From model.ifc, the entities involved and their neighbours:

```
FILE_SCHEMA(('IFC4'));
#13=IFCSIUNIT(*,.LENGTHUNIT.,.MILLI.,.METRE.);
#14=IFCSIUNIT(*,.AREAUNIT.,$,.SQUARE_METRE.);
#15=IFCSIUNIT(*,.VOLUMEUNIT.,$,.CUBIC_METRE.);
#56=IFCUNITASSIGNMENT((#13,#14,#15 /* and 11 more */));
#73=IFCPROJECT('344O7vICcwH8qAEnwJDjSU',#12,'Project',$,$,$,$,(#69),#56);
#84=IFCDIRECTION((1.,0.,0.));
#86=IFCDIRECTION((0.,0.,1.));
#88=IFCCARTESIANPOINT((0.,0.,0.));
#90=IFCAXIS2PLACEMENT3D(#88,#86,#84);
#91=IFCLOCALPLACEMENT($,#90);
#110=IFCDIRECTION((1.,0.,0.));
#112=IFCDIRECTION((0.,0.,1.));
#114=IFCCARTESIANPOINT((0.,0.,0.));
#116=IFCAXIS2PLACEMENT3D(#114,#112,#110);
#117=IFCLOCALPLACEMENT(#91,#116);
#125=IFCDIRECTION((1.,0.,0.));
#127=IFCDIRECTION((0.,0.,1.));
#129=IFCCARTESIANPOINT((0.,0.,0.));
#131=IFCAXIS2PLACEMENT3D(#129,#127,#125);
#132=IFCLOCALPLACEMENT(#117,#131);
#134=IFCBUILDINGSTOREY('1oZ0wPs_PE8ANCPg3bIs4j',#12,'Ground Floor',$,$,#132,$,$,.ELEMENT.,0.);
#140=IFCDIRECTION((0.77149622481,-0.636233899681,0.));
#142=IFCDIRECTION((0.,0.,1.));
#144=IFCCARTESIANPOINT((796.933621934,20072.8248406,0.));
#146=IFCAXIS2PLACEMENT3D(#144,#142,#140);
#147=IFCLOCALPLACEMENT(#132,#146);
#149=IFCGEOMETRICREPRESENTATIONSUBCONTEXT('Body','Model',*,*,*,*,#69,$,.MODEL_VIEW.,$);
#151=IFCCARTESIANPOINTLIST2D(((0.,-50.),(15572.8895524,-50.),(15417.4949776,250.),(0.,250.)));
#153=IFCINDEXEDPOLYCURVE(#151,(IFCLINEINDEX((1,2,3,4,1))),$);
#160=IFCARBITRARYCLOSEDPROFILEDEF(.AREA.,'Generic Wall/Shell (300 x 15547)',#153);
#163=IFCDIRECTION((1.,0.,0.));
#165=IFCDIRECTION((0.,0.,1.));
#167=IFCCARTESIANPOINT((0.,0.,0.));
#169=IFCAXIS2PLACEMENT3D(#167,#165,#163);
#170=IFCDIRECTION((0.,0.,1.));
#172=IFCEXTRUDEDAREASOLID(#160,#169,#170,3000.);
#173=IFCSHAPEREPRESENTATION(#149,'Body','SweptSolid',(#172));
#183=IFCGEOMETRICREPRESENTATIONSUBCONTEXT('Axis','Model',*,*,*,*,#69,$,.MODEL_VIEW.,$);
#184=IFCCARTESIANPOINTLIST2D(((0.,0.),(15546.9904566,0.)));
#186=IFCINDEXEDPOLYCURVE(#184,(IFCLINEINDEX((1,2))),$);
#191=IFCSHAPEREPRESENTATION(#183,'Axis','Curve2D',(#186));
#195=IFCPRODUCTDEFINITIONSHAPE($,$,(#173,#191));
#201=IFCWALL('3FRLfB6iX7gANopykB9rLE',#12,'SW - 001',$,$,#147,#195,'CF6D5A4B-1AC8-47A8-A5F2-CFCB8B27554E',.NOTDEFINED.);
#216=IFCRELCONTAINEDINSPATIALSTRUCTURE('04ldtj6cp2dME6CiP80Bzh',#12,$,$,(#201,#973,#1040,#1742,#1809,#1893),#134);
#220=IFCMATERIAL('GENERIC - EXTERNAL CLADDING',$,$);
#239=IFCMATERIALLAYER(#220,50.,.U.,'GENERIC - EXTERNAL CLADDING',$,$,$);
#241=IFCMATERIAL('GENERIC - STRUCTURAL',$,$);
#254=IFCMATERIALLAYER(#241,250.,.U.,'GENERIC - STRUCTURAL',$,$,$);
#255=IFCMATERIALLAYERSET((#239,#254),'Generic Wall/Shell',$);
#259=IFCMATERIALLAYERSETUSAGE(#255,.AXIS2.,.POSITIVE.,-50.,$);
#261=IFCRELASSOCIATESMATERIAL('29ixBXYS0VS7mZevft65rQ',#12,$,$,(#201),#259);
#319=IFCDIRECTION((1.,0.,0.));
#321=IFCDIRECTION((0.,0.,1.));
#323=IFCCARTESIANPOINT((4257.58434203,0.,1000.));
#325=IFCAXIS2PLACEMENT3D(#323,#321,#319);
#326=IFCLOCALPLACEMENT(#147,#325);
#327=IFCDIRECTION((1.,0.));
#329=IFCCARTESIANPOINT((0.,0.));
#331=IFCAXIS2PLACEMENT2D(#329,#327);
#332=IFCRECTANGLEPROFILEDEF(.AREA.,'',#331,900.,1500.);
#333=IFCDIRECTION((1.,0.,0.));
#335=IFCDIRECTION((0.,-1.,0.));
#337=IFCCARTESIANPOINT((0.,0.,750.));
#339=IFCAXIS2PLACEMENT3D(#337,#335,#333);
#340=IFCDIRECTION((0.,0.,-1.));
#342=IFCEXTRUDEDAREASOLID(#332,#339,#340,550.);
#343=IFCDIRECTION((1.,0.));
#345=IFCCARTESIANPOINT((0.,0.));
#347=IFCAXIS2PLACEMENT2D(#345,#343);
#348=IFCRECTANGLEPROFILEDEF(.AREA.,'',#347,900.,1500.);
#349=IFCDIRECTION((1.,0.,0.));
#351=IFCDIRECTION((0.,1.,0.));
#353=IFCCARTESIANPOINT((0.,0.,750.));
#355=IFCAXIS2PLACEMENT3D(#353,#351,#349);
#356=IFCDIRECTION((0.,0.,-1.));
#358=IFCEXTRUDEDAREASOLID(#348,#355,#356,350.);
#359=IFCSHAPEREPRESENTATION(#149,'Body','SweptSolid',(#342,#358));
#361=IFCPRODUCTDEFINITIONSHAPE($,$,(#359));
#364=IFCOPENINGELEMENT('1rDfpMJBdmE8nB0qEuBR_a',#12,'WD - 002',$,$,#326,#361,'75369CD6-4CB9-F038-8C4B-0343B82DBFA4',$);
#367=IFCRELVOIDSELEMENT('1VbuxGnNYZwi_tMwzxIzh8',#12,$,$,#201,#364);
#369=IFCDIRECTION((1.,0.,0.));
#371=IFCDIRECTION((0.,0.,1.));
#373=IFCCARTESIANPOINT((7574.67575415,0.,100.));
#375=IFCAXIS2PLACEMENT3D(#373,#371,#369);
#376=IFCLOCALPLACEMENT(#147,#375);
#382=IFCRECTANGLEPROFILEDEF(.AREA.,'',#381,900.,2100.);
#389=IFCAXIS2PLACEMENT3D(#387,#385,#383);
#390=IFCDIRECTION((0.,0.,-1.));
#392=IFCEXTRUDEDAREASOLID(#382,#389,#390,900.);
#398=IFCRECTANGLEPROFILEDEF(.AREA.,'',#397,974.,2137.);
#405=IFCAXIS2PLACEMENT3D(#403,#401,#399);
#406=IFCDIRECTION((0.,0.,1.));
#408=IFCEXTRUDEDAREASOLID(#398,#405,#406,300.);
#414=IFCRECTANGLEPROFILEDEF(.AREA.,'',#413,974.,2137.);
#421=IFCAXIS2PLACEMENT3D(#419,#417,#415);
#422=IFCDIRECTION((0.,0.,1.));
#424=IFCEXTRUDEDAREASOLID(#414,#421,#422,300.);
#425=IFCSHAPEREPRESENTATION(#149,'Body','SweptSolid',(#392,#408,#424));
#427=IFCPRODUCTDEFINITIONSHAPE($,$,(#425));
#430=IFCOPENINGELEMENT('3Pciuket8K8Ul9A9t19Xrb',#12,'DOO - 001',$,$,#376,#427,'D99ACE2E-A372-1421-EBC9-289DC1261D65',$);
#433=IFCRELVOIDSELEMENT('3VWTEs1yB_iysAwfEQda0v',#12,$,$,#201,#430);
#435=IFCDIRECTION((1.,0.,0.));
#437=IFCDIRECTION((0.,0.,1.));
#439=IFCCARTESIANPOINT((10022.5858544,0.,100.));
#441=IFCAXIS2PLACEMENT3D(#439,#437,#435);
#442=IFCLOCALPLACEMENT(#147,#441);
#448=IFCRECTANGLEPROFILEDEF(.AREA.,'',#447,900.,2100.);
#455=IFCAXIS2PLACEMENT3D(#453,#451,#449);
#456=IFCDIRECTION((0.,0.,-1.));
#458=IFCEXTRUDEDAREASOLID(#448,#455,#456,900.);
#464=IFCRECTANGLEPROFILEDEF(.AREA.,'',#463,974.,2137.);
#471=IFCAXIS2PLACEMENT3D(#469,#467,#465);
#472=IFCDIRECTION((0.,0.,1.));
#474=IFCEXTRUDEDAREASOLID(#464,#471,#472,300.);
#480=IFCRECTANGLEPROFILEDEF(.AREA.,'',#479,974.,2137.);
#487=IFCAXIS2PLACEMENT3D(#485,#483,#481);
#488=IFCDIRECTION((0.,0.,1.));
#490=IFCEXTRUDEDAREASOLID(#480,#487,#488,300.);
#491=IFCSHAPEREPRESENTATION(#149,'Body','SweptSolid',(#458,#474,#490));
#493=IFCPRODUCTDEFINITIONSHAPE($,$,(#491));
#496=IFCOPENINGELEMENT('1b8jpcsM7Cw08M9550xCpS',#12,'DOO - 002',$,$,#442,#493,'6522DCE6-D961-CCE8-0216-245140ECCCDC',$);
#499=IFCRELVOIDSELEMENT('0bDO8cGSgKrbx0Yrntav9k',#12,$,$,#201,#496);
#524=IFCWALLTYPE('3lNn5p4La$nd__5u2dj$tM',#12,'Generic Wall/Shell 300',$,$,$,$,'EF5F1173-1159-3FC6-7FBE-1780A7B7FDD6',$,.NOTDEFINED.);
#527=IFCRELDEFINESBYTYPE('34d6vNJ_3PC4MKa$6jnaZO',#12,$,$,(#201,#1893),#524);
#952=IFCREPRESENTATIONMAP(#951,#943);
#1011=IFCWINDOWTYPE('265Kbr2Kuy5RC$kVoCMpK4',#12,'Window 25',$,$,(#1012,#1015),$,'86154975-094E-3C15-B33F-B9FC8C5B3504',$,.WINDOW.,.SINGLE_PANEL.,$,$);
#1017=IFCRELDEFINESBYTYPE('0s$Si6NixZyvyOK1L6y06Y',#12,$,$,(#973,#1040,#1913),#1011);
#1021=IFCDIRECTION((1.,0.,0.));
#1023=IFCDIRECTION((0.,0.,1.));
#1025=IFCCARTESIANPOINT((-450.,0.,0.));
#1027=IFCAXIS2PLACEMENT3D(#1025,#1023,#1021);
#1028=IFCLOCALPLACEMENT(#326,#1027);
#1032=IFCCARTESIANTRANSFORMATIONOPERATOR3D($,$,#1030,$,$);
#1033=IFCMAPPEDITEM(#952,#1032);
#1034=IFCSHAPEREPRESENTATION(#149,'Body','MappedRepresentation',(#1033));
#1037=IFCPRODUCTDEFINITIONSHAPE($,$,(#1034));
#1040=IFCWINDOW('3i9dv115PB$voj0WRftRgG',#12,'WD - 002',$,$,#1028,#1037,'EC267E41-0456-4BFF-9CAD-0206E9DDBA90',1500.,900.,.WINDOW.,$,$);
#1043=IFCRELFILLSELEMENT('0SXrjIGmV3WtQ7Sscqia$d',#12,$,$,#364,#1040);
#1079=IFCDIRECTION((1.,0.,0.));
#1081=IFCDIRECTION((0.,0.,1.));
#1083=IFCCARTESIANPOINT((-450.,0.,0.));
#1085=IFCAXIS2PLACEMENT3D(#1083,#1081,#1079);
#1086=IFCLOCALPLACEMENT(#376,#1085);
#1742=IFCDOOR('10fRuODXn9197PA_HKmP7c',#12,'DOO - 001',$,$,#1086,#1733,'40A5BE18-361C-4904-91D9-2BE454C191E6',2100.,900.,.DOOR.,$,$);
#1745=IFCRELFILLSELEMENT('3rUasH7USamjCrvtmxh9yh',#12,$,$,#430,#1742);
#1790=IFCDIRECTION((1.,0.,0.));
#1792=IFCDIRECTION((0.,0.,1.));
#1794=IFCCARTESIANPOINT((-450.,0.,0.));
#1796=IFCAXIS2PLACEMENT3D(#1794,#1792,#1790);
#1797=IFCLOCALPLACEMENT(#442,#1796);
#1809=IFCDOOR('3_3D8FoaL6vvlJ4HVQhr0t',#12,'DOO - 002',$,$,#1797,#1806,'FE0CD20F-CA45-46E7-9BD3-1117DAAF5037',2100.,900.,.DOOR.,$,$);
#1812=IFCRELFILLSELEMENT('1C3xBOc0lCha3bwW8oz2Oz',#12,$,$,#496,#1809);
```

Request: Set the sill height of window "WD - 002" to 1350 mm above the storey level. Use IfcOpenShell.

```python
import numpy as np
import ifcopenshell
import ifcopenshell.api.geometry
import ifcopenshell.geom
import ifcopenshell.util.element
import ifcopenshell.util.placement
import ifcopenshell.util.shape
import ifcopenshell.util.unit

model = ifcopenshell.open("model.ifc")
unit_scale = ifcopenshell.util.unit.calculate_unit_scale(model)

window = model.by_guid("3i9dv115PB$voj0WRftRgG")
opening = window.FillsVoids[0].RelatingOpeningElement
storey = ifcopenshell.util.element.get_container(window, ifc_class="IfcBuildingStorey")
level = ifcopenshell.util.placement.get_local_placement(storey.ObjectPlacement)[2, 3]

# The opening's origin need not be at the sill, so measure its lowest point.
shape = ifcopenshell.geom.create_shape(ifcopenshell.geom.settings(), opening)
bottom = ifcopenshell.util.shape.get_shape_bottom_elevation(shape, shape.geometry) / unit_scale
dz = level + 1.35 / unit_scale - bottom

shift = np.array([0.0, 0.0, dz])
# The window is placed relative to its opening, so it follows when the opening moves.
matrix = ifcopenshell.util.placement.get_local_placement(opening.ObjectPlacement)
matrix[:3, 3] += shift
ifcopenshell.api.geometry.edit_object_placement(
    model, product=opening, matrix=matrix, is_si=False, should_transform_children=True
)

print(f"moved by {dz * unit_scale:+.3f} m")

model.write("model_updated.ifc")
```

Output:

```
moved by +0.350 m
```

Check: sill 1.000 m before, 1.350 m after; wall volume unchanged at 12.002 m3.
